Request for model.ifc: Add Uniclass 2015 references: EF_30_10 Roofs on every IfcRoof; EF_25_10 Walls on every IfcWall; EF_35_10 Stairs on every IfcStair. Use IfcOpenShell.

First a look at what the model holds.

```python
import ifcopenshell

model = ifcopenshell.open("model.ifc")
print(model.schema)
print("classifications:", [c.Name for c in model.by_type("IfcClassification")])
for ifc_class in ("IfcDoor", "IfcRoof", "IfcStair", "IfcWall", "IfcWindow"):
    print(ifc_class, len(model.by_type(ifc_class)))
```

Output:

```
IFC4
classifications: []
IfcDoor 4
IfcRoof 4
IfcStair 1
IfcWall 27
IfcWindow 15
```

```python
import ifcopenshell
import ifcopenshell.api.classification

model = ifcopenshell.open("model.ifc")

system = ifcopenshell.api.classification.add_classification(model, classification="Uniclass 2015")

codes = {
    "IfcRoof": ("EF_30_10", "Roofs"),
    "IfcWall": ("EF_25_10", "Walls"),
    "IfcStair": ("EF_35_10", "Stairs"),
}
for ifc_class, (code, name) in codes.items():
    products = model.by_type(ifc_class)
    ifcopenshell.api.classification.add_reference(
        model, products=products, classification=system, identification=code, name=name
    )
    print(code, len(products))

model.write("model_edited.ifc")
```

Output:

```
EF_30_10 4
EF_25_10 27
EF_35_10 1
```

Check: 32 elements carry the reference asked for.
